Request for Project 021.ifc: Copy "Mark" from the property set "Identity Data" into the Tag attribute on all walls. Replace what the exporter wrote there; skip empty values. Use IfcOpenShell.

First a look at what the model holds.

```python
import ifcopenshell
import ifcopenshell.util.element

model = ifcopenshell.open("Project 021.ifc")
print(model.schema)
walls = model.by_type("IfcWall")
print(len(walls), "walls")
for e in walls[:8]:
    source = ifcopenshell.util.element.get_pset(e, "Identity Data", "Mark")
    target = e.Tag
    print(e.id(), repr(source), repr(target), sep=" | ")
```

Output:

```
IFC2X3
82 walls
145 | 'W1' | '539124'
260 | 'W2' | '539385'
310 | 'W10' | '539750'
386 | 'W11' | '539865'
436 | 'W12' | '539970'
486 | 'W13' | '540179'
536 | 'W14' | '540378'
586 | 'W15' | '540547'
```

```python
import ifcopenshell
import ifcopenshell.util.element

model = ifcopenshell.open("Project 021.ifc")

count = 0
for e in model.by_type("IfcWall"):
    value = ifcopenshell.util.element.get_pset(e, "Identity Data", "Mark")
    current = e.Tag
    if not value or not value.strip() or current == value:
        continue
    e.Tag = value
    count += 1

print(count, "walls updated")

model.write("Project 021_edited.ifc")
```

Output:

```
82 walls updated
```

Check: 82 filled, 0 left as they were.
